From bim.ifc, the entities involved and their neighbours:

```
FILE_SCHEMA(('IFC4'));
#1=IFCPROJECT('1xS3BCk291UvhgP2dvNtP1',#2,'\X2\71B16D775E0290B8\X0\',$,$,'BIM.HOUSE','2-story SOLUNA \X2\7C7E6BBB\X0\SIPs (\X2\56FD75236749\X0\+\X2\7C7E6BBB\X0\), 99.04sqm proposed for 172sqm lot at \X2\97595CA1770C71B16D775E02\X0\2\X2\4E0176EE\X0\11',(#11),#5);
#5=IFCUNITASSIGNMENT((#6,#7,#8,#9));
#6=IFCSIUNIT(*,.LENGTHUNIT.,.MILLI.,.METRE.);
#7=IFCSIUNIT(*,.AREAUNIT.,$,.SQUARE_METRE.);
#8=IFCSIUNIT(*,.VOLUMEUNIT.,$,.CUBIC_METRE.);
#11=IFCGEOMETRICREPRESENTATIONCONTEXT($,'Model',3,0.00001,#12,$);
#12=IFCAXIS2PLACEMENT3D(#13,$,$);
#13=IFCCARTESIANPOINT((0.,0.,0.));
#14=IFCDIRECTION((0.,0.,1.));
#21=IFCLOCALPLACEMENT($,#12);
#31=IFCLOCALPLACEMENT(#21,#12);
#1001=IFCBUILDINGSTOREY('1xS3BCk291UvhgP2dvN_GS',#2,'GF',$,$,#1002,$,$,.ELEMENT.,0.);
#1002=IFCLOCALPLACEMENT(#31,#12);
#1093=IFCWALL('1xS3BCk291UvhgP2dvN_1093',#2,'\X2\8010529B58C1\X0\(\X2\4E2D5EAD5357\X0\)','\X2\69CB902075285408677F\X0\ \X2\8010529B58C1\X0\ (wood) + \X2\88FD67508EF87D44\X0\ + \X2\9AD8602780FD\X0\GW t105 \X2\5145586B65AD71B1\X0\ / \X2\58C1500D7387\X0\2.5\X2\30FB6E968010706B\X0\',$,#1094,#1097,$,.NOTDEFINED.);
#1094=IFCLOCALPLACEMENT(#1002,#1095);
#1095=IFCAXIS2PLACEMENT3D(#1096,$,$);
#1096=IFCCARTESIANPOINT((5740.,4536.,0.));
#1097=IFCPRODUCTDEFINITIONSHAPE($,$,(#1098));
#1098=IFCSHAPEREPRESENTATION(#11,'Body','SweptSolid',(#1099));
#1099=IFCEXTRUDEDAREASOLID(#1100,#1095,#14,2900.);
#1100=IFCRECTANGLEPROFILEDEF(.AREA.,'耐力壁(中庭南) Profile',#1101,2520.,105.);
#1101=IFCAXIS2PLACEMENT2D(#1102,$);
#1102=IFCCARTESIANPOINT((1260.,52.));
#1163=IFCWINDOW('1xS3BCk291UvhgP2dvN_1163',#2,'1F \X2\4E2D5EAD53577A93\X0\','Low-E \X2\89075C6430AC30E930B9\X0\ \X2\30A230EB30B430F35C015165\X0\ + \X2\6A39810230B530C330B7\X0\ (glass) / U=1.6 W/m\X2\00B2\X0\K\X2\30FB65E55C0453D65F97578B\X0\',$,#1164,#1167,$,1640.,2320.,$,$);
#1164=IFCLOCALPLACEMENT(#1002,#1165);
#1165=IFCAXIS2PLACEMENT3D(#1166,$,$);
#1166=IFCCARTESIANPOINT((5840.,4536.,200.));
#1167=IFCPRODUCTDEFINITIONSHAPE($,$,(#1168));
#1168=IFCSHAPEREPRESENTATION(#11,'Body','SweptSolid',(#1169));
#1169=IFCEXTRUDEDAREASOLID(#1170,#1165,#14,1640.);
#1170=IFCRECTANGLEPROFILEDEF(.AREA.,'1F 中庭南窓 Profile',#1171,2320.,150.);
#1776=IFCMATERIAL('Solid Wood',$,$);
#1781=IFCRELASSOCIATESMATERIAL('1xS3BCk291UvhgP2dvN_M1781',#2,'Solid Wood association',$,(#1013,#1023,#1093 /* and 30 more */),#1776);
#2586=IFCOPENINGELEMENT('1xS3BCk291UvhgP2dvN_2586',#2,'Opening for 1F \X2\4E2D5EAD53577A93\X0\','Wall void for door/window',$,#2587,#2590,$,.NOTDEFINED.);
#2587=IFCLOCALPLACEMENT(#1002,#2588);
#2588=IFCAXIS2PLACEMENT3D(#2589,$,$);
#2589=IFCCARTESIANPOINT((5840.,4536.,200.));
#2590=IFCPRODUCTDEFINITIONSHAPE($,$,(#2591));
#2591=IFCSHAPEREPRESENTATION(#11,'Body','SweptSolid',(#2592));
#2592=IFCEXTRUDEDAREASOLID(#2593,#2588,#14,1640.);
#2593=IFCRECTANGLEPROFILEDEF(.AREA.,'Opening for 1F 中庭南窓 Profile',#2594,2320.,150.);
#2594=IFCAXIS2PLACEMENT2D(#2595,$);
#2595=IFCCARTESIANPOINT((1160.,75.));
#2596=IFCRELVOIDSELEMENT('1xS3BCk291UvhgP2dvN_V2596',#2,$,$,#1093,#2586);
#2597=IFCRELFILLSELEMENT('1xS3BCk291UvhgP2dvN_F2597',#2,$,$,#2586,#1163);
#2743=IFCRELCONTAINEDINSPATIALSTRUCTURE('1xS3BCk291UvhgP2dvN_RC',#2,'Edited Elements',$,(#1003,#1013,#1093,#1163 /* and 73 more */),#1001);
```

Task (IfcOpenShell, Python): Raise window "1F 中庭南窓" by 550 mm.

```python
import numpy as np
import ifcopenshell
import ifcopenshell.api.geometry
import ifcopenshell.util.placement
import ifcopenshell.util.unit

model = ifcopenshell.open("bim.ifc")
unit_scale = ifcopenshell.util.unit.calculate_unit_scale(model)

window = model.by_guid("1xS3BCk291UvhgP2dvN_1163")
opening = window.FillsVoids[0].RelatingOpeningElement
dz = 550.0

shift = np.array([0.0, 0.0, dz])
# The window is not placed relative to its opening, so move both.
for product in (opening, window):
    matrix = ifcopenshell.util.placement.get_local_placement(product.ObjectPlacement)
    matrix[:3, 3] += shift
    ifcopenshell.api.geometry.edit_object_placement(model, product=product, matrix=matrix, is_si=False)

print(f"moved by {dz * unit_scale:+.3f} m")

model.write("bim_updated.ifc")
```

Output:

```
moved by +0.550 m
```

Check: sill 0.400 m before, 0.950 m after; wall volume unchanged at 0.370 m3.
